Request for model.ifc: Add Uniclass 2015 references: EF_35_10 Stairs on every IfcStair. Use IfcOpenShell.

First a look at what the model holds.

```python
import ifcopenshell

model = ifcopenshell.open("model.ifc")
print(model.schema)
print("classifications:", [c.Name for c in model.by_type("IfcClassification")])
for ifc_class in ("IfcDoor", "IfcRoof", "IfcStair", "IfcWall", "IfcWindow"):
    print(ifc_class, len(model.by_type(ifc_class)))
```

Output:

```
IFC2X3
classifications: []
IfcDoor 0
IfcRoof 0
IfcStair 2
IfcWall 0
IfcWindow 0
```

```python
import ifcopenshell
import ifcopenshell.api.classification

model = ifcopenshell.open("model.ifc")

# IFC2X3 requires Source and Edition and has no link from the project to the system.
system = model.create_entity("IfcClassification", Source="NBS", Edition="2015", Name="Uniclass 2015")

codes = {
    "IfcStair": ("EF_35_10", "Stairs"),
}
for ifc_class, (code, name) in codes.items():
    products = model.by_type(ifc_class)
    ifcopenshell.api.classification.add_reference(
        model, products=products, classification=system, identification=code, name=name
    )
    print(code, len(products))

model.write("model-out.ifc")
```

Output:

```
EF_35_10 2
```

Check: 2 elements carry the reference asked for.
